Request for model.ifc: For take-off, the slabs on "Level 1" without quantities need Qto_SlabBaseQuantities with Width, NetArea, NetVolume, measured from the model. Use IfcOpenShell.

First a look at what the model holds.

```python
import ifcopenshell
import ifcopenshell.util.element
import ifcopenshell.util.unit

model = ifcopenshell.open("model.ifc")
print(model.schema)
for unit_type in ("LENGTHUNIT", "AREAUNIT", "VOLUMEUNIT"):
    print(unit_type, ifcopenshell.util.unit.calculate_unit_scale(model, unit_type))
storey = next(s for s in model.by_type("IfcBuildingStorey") if s.Name == "Level 1")
slabs = [e for e in ifcopenshell.util.element.get_decomposition(storey) if e.is_a("IfcSlab")]
for e in sorted(slabs, key=lambda e: e.id()):
    print(e.id(), e.is_a(), e.Name, list(ifcopenshell.util.element.get_psets(e, qtos_only=True)), sep=" | ")
```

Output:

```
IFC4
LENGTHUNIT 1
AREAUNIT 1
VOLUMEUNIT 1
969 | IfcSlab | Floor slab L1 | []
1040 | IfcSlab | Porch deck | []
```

```python
import ifcopenshell
import ifcopenshell.api.pset
import ifcopenshell.geom
import ifcopenshell.util.element
import ifcopenshell.util.shape
import ifcopenshell.util.unit

model = ifcopenshell.open("model.ifc")
unit_scale = ifcopenshell.util.unit.calculate_unit_scale(model)
area_scale = ifcopenshell.util.unit.calculate_unit_scale(model, "AREAUNIT")
volume_scale = ifcopenshell.util.unit.calculate_unit_scale(model, "VOLUMEUNIT")
settings = ifcopenshell.geom.settings()

storey = next(s for s in model.by_type("IfcBuildingStorey") if s.Name == "Level 1")
slabs = [e for e in ifcopenshell.util.element.get_decomposition(storey) if e.is_a("IfcSlab")]

for e in sorted(slabs, key=lambda e: e.id()):
    if ifcopenshell.util.element.get_psets(e, qtos_only=True, should_inherit=False):
        continue
    # Geometry comes back in metres, in the element's own axes.
    shape = ifcopenshell.geom.create_shape(settings, e)
    values = {
        "Width": ifcopenshell.util.shape.get_z(shape.geometry) / unit_scale,
        "NetArea": ifcopenshell.util.shape.get_footprint_area(shape.geometry) / area_scale,
        "NetVolume": ifcopenshell.util.shape.get_volume(shape.geometry) / volume_scale,
    }
    qto = ifcopenshell.api.pset.add_qto(model, product=e, name="Qto_SlabBaseQuantities")
    ifcopenshell.api.pset.edit_qto(model, qto=qto, properties=values)
    print(e.id(), {k: round(v, 3) for k, v in values.items()})

model.write("model_edited.ifc")
```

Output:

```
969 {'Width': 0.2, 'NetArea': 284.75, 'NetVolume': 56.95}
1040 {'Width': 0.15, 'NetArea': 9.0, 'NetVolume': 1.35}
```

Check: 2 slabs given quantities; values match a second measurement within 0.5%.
